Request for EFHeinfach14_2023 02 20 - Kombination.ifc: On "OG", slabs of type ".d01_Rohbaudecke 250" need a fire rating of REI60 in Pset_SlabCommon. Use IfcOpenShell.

First a look at what the model holds.

```python
import ifcopenshell
import ifcopenshell.util.element

model = ifcopenshell.open("EFHeinfach14_2023 02 20 - Kombination.ifc")
print(model.schema)
storey = next(s for s in model.by_type("IfcBuildingStorey") if s.Name == "OG")
slabs = [e for e in ifcopenshell.util.element.get_decomposition(storey) if e.is_a("IfcSlab")]
seen = {}
for e in slabs:
    element_type = ifcopenshell.util.element.get_type(e)
    key = (element_type.Name if element_type != e and element_type else None, ifcopenshell.util.element.get_pset(e, "Pset_SlabCommon", "FireRating"))
    seen[key] = seen.get(key, 0) + 1
for (name, value), count in sorted(seen.items(), key=str):
    print(count, "x", name, "|", value)
```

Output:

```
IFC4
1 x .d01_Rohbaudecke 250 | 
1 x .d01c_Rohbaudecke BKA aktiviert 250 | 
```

```python
import ifcopenshell
import ifcopenshell.api.pset
import ifcopenshell.util.element

model = ifcopenshell.open("EFHeinfach14_2023 02 20 - Kombination.ifc")

storey = next(s for s in model.by_type("IfcBuildingStorey") if s.Name == "OG")
slabs = [e for e in ifcopenshell.util.element.get_decomposition(storey) if e.is_a("IfcSlab")]

count = 0
for e in slabs:
    element_type = ifcopenshell.util.element.get_type(e)
    if element_type in (None, e) or element_type.Name != ".d01_Rohbaudecke 250":
        continue
    # add_pset returns the element's existing set when there is one.
    pset = ifcopenshell.api.pset.add_pset(model, product=e, name="Pset_SlabCommon")
    ifcopenshell.api.pset.edit_pset(model, pset=pset, properties={"FireRating": "REI60"})
    count += 1

print(count, "slabs updated")

model.write("EFHeinfach14_2023 02 20 - Kombination_rev.ifc")
```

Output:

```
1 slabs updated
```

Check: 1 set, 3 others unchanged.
